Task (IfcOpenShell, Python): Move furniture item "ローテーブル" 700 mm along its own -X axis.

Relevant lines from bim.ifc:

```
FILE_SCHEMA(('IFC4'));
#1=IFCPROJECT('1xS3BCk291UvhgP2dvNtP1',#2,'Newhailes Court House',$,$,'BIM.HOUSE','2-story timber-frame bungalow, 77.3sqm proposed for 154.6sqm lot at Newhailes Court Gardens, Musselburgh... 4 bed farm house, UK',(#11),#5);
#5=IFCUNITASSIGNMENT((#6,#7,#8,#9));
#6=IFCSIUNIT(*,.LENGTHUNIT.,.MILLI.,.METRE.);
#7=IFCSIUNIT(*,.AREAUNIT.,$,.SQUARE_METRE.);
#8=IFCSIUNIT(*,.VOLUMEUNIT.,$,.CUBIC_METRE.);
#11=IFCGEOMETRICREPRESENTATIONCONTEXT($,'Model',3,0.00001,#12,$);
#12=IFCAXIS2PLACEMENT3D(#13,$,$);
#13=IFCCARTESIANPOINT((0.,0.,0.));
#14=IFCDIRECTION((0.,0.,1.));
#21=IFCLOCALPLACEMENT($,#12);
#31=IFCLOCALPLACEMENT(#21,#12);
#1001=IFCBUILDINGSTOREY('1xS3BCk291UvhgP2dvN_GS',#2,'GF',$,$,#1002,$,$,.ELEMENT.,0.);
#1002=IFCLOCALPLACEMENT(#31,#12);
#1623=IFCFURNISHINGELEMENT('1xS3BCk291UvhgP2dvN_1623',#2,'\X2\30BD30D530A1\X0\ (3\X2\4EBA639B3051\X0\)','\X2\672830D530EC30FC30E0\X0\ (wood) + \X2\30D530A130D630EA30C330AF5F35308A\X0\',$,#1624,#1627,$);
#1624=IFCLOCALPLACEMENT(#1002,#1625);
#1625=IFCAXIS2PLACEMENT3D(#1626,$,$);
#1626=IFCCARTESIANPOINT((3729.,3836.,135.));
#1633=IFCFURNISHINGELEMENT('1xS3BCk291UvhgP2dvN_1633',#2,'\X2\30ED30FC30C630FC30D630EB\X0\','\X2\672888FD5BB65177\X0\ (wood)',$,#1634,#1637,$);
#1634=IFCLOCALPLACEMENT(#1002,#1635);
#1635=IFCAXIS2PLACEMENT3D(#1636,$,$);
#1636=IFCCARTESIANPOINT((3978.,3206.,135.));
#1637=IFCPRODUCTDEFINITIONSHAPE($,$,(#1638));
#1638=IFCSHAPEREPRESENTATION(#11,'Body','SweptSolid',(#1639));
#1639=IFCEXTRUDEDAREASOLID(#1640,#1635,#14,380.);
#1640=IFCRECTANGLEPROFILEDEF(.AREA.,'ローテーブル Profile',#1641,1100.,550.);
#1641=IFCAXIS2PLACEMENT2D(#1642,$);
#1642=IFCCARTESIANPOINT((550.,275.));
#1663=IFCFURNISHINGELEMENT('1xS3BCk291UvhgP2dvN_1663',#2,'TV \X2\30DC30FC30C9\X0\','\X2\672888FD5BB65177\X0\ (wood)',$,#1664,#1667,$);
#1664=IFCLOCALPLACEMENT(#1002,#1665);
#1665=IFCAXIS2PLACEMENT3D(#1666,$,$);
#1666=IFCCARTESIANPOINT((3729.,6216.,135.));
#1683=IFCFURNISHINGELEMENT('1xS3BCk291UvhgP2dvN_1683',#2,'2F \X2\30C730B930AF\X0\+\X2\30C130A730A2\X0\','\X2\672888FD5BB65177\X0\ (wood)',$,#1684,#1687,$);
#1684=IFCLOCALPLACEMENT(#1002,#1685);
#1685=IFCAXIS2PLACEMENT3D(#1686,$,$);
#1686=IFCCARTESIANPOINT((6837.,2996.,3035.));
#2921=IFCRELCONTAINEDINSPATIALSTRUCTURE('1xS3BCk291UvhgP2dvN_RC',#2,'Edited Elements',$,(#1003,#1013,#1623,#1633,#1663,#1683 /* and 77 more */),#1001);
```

```python
import ifcopenshell
import ifcopenshell.api.geometry
import ifcopenshell.util.placement

model = ifcopenshell.open("bim.ifc")

item = model.by_guid("1xS3BCk291UvhgP2dvN_1633")
matrix = ifcopenshell.util.placement.get_local_placement(item.ObjectPlacement)
matrix[:3, 3] -= matrix[:3, 0] * 700.0
ifcopenshell.api.geometry.edit_object_placement(model, product=item, matrix=matrix, is_si=False)

print(ifcopenshell.util.placement.get_local_placement(item.ObjectPlacement).round(3) + 0.0)

model.write("bim_edited.ifc")
```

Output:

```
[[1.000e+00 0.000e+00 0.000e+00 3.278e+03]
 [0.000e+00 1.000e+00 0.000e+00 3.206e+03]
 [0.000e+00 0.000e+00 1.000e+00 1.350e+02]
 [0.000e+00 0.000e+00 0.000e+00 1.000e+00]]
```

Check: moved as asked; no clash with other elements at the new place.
